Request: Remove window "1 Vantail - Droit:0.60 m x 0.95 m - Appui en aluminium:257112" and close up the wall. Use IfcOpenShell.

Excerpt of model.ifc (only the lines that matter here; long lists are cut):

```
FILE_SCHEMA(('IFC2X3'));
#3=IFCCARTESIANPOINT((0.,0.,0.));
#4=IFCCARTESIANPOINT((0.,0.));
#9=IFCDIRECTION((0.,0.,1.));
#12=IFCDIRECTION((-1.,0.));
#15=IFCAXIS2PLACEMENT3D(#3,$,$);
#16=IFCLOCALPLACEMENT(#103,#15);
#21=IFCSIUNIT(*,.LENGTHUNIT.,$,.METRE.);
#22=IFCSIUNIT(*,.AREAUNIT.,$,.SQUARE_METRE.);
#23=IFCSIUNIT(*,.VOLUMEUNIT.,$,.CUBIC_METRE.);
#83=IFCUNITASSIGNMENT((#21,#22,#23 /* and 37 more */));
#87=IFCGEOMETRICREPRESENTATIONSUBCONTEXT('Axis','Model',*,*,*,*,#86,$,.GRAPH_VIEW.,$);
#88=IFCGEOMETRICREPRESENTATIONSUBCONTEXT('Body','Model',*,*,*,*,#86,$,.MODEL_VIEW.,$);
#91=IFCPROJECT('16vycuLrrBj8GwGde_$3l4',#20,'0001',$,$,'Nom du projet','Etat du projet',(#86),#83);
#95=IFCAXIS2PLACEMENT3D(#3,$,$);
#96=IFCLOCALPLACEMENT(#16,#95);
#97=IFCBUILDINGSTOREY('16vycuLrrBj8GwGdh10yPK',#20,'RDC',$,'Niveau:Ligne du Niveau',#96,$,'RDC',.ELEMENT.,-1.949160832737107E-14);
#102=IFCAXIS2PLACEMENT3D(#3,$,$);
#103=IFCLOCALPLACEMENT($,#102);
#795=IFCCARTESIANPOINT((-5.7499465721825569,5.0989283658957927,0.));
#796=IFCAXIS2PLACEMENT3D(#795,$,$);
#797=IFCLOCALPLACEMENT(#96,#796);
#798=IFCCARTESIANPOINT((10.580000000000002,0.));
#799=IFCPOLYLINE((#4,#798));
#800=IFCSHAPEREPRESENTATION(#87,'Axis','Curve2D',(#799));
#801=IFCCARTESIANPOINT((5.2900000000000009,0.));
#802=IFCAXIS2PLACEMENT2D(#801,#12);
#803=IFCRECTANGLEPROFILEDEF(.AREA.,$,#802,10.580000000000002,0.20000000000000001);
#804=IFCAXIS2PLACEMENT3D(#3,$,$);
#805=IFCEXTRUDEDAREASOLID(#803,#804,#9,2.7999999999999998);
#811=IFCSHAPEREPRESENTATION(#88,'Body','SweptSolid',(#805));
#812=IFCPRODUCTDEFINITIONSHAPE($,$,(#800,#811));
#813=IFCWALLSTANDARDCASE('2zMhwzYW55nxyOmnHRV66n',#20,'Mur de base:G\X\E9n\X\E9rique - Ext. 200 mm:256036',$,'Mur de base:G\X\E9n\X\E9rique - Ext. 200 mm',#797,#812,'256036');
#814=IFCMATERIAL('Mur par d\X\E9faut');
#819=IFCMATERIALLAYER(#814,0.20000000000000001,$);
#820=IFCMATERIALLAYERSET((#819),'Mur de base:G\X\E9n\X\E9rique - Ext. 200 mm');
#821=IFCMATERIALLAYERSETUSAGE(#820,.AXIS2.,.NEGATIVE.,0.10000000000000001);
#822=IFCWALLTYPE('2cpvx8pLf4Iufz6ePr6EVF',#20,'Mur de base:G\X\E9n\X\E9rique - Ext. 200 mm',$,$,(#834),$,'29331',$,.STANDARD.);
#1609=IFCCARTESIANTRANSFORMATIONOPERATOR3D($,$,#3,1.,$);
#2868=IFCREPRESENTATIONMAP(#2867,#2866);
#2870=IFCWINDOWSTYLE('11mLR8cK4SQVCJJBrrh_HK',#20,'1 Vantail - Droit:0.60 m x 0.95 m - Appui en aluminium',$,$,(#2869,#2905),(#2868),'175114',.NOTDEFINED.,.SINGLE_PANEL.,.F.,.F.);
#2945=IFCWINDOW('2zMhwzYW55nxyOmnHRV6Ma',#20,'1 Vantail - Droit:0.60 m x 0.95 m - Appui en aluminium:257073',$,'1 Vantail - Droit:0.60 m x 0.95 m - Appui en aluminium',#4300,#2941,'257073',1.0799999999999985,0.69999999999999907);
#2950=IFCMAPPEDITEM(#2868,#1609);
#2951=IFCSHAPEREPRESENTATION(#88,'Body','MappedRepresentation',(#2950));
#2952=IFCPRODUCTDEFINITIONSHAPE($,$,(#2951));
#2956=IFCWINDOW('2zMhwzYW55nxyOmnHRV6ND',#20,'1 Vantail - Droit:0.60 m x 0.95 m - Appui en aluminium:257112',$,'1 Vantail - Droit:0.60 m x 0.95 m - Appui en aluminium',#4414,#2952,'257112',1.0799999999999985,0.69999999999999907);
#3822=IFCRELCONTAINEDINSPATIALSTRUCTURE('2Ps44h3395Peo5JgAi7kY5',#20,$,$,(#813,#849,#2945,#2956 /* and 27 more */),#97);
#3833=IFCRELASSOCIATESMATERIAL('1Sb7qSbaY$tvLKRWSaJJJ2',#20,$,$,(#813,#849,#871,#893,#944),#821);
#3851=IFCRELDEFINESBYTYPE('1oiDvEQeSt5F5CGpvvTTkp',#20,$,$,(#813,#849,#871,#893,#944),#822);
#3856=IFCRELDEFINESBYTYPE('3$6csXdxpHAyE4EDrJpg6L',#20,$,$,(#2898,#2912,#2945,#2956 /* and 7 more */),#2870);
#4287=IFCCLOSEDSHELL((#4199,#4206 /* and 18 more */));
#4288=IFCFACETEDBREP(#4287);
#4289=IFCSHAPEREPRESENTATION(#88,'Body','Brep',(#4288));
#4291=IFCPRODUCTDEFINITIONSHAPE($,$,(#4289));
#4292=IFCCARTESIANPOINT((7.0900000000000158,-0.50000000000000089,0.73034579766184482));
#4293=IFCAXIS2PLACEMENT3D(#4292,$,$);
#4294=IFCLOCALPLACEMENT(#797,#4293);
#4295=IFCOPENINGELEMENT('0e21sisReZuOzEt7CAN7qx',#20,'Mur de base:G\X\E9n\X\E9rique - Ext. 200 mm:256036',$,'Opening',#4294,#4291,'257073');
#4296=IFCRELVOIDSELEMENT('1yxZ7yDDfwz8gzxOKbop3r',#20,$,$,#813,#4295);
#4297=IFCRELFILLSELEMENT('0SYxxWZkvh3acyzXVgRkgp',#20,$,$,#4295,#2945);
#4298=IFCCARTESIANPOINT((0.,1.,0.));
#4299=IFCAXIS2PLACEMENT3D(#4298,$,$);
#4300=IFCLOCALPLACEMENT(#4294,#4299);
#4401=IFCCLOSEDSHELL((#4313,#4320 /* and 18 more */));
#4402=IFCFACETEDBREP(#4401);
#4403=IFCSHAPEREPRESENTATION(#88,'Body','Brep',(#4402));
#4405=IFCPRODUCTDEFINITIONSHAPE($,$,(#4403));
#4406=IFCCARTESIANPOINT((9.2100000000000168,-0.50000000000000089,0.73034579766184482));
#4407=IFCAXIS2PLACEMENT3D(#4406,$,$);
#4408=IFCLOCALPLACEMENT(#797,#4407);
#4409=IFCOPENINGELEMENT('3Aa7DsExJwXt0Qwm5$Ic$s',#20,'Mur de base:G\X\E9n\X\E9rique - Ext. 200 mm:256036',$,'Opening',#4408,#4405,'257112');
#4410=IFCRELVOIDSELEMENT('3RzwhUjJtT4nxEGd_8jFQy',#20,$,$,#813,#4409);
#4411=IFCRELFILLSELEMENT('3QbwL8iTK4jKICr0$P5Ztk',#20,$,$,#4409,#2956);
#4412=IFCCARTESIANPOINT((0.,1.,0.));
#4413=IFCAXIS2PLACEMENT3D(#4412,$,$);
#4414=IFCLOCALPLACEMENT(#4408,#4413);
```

```python
import ifcopenshell
import ifcopenshell.api.feature
import ifcopenshell.api.root
import ifcopenshell.geom
import ifcopenshell.util.shape

model = ifcopenshell.open("model.ifc")
settings = ifcopenshell.geom.settings()


def volume(element):
    """Net volume in cubic metres, openings subtracted."""
    shape = ifcopenshell.geom.create_shape(settings, element)
    return ifcopenshell.util.shape.get_volume(shape.geometry)


window = model.by_guid("2zMhwzYW55nxyOmnHRV6ND")
opening = window.FillsVoids[0].RelatingOpeningElement
wall = opening.VoidsElements[0].RelatingBuildingElement
before = volume(wall)

ifcopenshell.api.root.remove_product(model, product=window)
ifcopenshell.api.feature.remove_feature(model, feature=opening)

after = volume(wall)

print(f"wall volume {before:.3f} -> {after:.3f} m3")

model.write("model_updated.ifc")
```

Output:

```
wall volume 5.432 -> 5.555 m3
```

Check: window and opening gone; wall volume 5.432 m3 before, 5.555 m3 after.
